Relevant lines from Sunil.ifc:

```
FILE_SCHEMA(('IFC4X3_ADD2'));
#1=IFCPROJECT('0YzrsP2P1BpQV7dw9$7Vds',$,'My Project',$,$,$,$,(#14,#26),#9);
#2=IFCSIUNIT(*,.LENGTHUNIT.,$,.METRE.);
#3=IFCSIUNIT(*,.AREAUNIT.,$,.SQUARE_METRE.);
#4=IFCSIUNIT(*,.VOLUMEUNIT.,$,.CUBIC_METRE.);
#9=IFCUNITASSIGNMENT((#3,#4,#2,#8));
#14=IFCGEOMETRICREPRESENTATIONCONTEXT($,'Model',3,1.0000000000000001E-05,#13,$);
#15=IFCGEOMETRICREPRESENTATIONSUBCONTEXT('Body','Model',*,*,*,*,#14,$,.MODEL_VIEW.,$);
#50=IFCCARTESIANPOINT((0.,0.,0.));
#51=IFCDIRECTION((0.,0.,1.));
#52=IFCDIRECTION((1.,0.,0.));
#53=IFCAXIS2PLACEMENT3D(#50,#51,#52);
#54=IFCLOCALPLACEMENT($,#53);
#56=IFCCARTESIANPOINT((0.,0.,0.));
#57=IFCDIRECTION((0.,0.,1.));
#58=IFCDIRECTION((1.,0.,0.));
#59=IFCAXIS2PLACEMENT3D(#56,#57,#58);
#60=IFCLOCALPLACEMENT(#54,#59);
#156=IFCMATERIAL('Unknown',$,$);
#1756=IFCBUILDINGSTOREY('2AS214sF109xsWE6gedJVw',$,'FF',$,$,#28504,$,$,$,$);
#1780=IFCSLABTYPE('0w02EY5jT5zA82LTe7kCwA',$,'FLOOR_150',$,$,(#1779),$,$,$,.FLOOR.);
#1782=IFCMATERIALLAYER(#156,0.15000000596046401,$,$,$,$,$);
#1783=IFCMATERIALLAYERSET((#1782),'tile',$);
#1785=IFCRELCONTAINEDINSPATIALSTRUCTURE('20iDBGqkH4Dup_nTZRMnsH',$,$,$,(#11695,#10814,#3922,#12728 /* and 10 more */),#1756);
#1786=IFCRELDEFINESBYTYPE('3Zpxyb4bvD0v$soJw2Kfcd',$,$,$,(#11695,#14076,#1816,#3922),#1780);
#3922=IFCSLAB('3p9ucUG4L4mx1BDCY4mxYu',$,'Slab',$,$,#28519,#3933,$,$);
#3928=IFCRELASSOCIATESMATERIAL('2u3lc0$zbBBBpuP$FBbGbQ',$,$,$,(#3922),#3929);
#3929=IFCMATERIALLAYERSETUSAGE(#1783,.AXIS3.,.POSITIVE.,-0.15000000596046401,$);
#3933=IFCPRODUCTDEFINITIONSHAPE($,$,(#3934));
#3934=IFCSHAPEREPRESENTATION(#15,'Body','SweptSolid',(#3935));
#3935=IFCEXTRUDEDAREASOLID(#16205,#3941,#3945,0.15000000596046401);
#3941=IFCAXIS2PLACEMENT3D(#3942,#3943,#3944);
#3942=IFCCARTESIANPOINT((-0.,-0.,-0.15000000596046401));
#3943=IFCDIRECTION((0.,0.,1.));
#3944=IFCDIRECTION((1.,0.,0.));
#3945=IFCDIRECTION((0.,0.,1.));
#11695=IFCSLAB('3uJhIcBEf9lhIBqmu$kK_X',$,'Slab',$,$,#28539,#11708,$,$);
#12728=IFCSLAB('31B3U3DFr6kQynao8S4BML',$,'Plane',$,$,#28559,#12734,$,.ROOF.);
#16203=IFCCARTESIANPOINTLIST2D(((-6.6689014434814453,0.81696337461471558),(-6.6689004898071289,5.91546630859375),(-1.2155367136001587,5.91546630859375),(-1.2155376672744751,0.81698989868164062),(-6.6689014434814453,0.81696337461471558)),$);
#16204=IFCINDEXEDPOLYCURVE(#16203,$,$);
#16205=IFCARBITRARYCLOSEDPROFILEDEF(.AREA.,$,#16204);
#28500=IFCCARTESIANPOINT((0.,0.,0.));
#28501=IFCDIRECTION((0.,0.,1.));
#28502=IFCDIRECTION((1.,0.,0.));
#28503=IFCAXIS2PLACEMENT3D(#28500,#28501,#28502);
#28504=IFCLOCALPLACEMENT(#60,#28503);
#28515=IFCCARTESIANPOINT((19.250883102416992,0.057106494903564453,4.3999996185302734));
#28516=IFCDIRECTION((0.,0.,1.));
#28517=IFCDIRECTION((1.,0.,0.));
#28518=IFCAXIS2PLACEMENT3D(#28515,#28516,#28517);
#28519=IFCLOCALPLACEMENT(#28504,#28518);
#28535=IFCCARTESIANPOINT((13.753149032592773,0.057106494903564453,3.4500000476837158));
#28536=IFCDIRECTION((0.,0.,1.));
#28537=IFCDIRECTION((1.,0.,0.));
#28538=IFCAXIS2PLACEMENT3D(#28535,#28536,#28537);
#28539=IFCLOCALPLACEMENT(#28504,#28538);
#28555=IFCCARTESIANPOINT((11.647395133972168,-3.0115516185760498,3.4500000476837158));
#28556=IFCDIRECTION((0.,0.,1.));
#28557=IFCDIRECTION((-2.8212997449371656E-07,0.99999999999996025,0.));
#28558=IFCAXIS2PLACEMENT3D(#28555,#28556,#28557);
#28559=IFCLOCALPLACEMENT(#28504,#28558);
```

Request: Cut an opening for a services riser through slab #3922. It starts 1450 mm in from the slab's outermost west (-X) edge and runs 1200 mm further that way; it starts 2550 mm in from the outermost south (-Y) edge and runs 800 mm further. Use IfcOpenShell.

```python
import numpy as np
import ifcopenshell
import ifcopenshell.api.feature
import ifcopenshell.api.geometry
import ifcopenshell.api.root
import ifcopenshell.geom
import ifcopenshell.util.placement
import ifcopenshell.util.representation
import ifcopenshell.util.shape
import ifcopenshell.util.unit

model = ifcopenshell.open("Sunil.ifc")
unit_scale = ifcopenshell.util.unit.calculate_unit_scale(model)
settings = ifcopenshell.geom.settings()


def volume(element):
    """Net volume in cubic metres, openings subtracted."""
    shape = ifcopenshell.geom.create_shape(settings, element)
    return ifcopenshell.util.shape.get_volume(shape.geometry)


slab = model.by_id(3922)
before = volume(slab)

# Extent in the slab's own axes, in metres. The edges named are its -X and -Y sides.
slab_shape = ifcopenshell.geom.create_shape(settings, slab)
vertices = ifcopenshell.util.shape.get_vertices(slab_shape.geometry)
x_min, y_min, bottom = vertices.min(axis=0)
top = vertices[:, 2].max()

opening = ifcopenshell.api.root.create_entity(model, ifc_class="IfcOpeningElement", name="Services riser opening", predefined_type="OPENING")
context = ifcopenshell.util.representation.get_context(model, "Model", "Body", "MODEL_VIEW")
width, depth = 1.2, 0.8
outline = [(0.0, 0.0), (width, 0.0), (width, depth), (0.0, depth), (0.0, 0.0)]
# Overshoot both faces by 50 mm so the cut is clean.
shape = ifcopenshell.api.geometry.add_slab_representation(
    model, context=context, depth=top - bottom + 0.1, polyline=outline
)
ifcopenshell.api.geometry.assign_representation(model, product=opening, representation=shape)

matrix = ifcopenshell.util.placement.get_local_placement(slab.ObjectPlacement)
matrix[:, 3] = matrix @ np.append(np.array([x_min + 1.45, y_min + 2.55, bottom - 0.05]) / unit_scale, 1.0)
ifcopenshell.api.geometry.edit_object_placement(model, product=opening, matrix=matrix, is_si=False)
ifcopenshell.api.feature.add_feature(model, feature=opening, element=slab)

after = volume(slab)

print(f"slab volume {before:.3f} -> {after:.3f} m3")

model.write("Sunil_v2.ifc")
```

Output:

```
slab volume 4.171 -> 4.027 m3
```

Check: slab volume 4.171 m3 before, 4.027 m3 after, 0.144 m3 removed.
